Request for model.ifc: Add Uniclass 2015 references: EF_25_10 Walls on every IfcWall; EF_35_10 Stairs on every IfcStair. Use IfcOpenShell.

First a look at what the model holds.

```python
import ifcopenshell

model = ifcopenshell.open("model.ifc")
print(model.schema)
print("classifications:", [c.Name for c in model.by_type("IfcClassification")])
for ifc_class in ("IfcDoor", "IfcRoof", "IfcStair", "IfcWall", "IfcWindow"):
    print(ifc_class, len(model.by_type(ifc_class)))
```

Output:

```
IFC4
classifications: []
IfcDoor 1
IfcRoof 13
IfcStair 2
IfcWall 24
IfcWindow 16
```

```python
import ifcopenshell
import ifcopenshell.api.classification

model = ifcopenshell.open("model.ifc")

system = ifcopenshell.api.classification.add_classification(model, classification="Uniclass 2015")

codes = {
    "IfcWall": ("EF_25_10", "Walls"),
    "IfcStair": ("EF_35_10", "Stairs"),
}
for ifc_class, (code, name) in codes.items():
    products = model.by_type(ifc_class)
    ifcopenshell.api.classification.add_reference(
        model, products=products, classification=system, identification=code, name=name
    )
    print(code, len(products))

model.write("model_edited.ifc")
```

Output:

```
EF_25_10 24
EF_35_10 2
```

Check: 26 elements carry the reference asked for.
